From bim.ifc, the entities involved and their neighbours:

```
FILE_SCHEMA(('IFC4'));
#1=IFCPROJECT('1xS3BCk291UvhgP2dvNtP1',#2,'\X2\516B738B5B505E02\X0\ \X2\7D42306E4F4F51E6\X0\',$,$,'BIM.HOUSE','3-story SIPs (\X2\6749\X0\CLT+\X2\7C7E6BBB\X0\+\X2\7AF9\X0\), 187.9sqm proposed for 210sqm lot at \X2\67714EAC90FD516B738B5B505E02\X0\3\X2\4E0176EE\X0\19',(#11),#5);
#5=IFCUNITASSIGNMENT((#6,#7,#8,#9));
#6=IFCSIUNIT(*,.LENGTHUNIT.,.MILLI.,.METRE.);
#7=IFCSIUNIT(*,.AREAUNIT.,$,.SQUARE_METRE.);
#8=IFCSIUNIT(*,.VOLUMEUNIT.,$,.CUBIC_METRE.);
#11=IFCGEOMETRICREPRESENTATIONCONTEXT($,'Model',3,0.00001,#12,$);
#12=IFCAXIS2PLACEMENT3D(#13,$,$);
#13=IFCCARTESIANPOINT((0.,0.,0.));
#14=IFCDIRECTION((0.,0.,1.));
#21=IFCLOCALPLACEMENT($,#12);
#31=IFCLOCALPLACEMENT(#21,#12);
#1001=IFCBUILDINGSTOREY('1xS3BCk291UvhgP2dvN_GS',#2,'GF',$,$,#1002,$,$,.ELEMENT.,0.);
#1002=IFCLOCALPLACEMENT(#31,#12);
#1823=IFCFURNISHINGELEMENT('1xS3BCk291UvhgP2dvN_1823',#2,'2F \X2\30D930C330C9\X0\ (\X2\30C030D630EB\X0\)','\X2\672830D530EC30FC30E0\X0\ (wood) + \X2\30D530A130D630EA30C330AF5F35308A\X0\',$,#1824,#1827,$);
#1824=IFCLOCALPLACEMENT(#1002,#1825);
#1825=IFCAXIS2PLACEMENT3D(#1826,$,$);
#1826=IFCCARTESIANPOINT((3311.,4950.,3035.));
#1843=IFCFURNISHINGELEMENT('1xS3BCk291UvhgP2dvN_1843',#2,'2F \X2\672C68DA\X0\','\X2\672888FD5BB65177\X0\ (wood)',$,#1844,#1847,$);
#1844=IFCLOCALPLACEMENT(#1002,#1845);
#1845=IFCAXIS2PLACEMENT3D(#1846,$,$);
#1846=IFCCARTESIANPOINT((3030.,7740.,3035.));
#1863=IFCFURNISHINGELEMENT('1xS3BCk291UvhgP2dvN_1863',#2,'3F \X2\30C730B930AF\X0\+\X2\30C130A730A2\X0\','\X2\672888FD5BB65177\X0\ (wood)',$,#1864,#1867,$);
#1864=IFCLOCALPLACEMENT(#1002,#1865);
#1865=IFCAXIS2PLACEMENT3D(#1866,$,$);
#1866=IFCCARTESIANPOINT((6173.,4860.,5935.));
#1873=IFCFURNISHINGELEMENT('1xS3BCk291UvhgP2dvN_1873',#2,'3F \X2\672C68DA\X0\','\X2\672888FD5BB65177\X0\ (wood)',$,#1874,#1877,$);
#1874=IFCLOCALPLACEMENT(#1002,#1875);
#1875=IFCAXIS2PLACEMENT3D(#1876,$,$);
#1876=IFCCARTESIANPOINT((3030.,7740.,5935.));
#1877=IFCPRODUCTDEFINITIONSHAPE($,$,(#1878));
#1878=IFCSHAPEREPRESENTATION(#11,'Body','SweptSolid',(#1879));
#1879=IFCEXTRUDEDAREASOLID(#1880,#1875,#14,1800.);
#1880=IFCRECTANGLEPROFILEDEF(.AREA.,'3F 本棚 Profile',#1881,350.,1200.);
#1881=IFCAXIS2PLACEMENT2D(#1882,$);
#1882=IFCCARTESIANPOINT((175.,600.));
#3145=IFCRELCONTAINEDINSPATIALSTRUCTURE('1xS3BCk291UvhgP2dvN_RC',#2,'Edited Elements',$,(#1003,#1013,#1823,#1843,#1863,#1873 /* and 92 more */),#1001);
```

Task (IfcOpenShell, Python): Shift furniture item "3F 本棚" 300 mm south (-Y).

```python
import ifcopenshell
import ifcopenshell.api.geometry
import ifcopenshell.util.placement

model = ifcopenshell.open("bim.ifc")

item = model.by_id(1873)
matrix = ifcopenshell.util.placement.get_local_placement(item.ObjectPlacement)
matrix[1, 3] -= 300.0
ifcopenshell.api.geometry.edit_object_placement(model, product=item, matrix=matrix, is_si=False)

print(ifcopenshell.util.placement.get_local_placement(item.ObjectPlacement).round(3) + 0.0)

model.write("bim-out.ifc")
```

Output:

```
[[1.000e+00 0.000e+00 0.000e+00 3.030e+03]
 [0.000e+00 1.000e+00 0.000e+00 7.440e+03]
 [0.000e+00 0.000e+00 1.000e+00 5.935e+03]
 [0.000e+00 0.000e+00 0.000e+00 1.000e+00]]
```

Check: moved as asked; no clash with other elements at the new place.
